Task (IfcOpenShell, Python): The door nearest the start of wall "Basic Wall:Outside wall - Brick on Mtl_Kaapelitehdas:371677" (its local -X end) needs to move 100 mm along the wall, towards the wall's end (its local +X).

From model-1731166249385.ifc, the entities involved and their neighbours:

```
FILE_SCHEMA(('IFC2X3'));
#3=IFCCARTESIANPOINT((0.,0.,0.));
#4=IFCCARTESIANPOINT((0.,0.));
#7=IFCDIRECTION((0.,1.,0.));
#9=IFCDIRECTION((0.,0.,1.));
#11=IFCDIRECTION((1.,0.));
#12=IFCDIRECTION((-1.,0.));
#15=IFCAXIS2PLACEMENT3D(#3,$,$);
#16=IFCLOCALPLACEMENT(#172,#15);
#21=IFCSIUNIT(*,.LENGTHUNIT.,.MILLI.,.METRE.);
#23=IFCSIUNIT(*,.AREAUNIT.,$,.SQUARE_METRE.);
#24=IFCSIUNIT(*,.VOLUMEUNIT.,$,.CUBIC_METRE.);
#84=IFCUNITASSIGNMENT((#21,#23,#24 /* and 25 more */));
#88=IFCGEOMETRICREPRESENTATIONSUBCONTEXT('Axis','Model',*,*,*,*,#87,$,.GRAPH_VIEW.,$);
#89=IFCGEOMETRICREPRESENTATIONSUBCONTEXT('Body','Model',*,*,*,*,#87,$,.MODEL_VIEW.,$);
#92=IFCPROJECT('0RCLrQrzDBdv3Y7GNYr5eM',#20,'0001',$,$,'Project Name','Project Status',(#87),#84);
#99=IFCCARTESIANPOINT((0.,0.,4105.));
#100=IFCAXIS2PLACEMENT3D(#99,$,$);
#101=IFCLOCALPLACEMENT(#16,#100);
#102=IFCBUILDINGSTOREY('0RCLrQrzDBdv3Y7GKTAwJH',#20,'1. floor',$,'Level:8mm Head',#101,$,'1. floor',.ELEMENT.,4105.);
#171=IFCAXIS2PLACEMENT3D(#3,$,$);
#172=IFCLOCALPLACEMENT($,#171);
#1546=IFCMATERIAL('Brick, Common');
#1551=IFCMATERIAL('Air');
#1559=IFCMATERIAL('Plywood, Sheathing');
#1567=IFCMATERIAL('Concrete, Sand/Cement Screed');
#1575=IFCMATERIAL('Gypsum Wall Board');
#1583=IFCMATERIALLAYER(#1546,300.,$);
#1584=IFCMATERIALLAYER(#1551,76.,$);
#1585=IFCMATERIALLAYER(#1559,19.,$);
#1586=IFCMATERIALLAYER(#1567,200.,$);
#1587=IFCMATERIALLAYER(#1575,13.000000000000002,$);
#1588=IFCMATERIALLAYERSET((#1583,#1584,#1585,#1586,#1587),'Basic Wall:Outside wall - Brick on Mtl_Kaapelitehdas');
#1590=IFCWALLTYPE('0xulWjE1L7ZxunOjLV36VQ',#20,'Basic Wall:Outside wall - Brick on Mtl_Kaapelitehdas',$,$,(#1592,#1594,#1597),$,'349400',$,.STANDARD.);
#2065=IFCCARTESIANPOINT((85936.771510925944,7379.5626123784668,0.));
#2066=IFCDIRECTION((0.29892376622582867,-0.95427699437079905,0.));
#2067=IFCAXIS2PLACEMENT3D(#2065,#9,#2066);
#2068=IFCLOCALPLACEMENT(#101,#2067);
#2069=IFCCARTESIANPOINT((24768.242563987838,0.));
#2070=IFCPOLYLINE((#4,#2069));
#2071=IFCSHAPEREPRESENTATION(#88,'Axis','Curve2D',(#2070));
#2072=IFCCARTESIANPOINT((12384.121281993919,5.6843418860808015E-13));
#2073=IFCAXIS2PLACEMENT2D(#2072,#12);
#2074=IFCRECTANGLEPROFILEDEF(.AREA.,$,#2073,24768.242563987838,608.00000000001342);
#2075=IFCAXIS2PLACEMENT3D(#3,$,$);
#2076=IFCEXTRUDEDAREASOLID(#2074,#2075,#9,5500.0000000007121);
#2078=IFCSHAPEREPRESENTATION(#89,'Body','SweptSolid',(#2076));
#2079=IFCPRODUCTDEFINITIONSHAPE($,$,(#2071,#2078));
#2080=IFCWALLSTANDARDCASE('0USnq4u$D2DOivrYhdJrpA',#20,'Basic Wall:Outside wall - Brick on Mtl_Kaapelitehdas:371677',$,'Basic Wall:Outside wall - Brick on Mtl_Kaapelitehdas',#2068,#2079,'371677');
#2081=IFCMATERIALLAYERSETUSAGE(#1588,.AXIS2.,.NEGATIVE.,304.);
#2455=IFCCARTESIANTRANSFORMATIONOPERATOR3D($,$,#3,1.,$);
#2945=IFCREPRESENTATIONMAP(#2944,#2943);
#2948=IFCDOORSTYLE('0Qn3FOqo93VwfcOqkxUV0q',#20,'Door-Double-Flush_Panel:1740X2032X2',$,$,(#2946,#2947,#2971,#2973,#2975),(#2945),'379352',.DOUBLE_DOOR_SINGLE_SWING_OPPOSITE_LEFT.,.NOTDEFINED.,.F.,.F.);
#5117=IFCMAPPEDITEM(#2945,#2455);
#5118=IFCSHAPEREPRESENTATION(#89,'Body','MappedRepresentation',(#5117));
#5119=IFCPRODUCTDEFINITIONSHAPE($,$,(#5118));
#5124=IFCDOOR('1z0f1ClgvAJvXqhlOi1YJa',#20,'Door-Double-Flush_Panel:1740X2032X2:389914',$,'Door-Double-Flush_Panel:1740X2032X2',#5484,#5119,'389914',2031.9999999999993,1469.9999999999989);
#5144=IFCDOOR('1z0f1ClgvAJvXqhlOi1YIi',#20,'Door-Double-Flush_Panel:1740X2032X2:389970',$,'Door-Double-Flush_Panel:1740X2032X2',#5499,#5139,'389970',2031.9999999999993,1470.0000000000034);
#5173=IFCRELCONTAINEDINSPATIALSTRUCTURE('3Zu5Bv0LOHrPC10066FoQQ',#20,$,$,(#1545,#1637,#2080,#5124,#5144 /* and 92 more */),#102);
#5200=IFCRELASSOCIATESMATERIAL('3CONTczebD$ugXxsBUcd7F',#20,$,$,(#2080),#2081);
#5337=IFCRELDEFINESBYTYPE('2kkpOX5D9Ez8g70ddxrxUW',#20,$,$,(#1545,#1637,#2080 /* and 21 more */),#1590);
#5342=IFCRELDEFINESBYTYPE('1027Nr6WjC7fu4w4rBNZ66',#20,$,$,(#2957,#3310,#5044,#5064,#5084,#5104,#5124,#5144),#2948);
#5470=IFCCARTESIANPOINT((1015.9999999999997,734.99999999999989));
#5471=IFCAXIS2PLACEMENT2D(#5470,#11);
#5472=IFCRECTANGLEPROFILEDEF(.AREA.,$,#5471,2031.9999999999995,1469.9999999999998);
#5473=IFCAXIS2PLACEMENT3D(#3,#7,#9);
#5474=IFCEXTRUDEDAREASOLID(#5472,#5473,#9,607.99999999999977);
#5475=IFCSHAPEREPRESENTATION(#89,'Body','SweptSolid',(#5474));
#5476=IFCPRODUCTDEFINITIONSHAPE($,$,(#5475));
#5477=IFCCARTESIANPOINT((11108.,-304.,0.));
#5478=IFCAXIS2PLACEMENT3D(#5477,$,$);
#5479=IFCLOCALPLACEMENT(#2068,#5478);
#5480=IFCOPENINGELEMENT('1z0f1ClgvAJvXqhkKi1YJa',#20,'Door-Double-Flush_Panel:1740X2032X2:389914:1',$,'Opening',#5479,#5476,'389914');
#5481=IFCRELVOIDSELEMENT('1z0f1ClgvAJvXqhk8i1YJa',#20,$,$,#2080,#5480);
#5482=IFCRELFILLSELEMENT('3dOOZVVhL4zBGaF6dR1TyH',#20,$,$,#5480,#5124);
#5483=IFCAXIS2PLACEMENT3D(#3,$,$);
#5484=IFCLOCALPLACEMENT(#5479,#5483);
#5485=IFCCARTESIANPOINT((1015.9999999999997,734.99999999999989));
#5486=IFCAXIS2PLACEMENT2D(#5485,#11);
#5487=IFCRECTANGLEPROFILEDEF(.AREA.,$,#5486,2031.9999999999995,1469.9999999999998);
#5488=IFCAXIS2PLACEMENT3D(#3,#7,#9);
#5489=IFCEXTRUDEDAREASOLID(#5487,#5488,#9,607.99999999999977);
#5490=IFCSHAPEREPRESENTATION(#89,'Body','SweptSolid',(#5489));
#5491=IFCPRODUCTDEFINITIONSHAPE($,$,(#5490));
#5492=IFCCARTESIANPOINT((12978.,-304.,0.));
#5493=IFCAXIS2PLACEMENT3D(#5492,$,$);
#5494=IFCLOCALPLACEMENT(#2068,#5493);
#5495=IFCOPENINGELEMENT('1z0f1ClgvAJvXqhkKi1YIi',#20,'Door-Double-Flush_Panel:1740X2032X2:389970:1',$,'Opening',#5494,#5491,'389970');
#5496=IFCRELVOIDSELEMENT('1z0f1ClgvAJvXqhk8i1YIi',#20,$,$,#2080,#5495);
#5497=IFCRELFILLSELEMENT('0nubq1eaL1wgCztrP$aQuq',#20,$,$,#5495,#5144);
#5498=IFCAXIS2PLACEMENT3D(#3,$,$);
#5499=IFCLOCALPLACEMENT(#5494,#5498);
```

```python
import ifcopenshell
import ifcopenshell.api.geometry
import ifcopenshell.util.placement

model = ifcopenshell.open("model-1731166249385.ifc")

door = model.by_id(5124)
opening = door.FillsVoids[0].RelatingOpeningElement
wall = opening.VoidsElements[0].RelatingBuildingElement

wall_matrix = ifcopenshell.util.placement.get_local_placement(wall.ObjectPlacement)
shift = wall_matrix[:3, 0] * 100.0
before = ifcopenshell.util.placement.get_local_placement(door.ObjectPlacement)[:3, 3].copy()

# The door is placed relative to its opening, so it follows when the opening moves.
matrix = ifcopenshell.util.placement.get_local_placement(opening.ObjectPlacement)
matrix[:3, 3] += shift
ifcopenshell.api.geometry.edit_object_placement(
    model, product=opening, matrix=matrix, is_si=False, should_transform_children=True
)

after = ifcopenshell.util.placement.get_local_placement(door.ObjectPlacement)[:3, 3]
print("door moved by", (after - before).round(3) + 0.0)

model.write("model-1731166249385_updated.ifc")
```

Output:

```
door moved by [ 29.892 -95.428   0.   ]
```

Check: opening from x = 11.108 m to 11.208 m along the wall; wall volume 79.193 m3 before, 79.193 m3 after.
